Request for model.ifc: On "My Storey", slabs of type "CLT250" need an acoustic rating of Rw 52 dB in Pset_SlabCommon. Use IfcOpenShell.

First a look at what the model holds.

```python
import ifcopenshell
import ifcopenshell.util.element

model = ifcopenshell.open("model.ifc")
print(model.schema)
storey = next(s for s in model.by_type("IfcBuildingStorey") if s.Name == "My Storey")
slabs = [e for e in ifcopenshell.util.element.get_decomposition(storey) if e.is_a("IfcSlab")]
seen = {}
for e in slabs:
    element_type = ifcopenshell.util.element.get_type(e)
    key = (element_type.Name if element_type != e and element_type else None, ifcopenshell.util.element.get_pset(e, "Pset_SlabCommon", "AcousticRating"))
    seen[key] = seen.get(key, 0) + 1
for (name, value), count in sorted(seen.items(), key=str):
    print(count, "x", name, "|", value)
```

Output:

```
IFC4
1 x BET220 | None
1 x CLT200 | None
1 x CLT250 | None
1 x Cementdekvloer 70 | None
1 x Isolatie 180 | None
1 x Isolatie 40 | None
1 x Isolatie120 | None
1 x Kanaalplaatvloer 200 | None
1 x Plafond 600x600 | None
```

```python
import ifcopenshell
import ifcopenshell.api.pset
import ifcopenshell.util.element

model = ifcopenshell.open("model.ifc")

storey = next(s for s in model.by_type("IfcBuildingStorey") if s.Name == "My Storey")
slabs = [e for e in ifcopenshell.util.element.get_decomposition(storey) if e.is_a("IfcSlab")]

count = 0
for e in slabs:
    element_type = ifcopenshell.util.element.get_type(e)
    if element_type in (None, e) or element_type.Name != "CLT250":
        continue
    # add_pset returns the element's existing set when there is one.
    pset = ifcopenshell.api.pset.add_pset(model, product=e, name="Pset_SlabCommon")
    ifcopenshell.api.pset.edit_pset(model, pset=pset, properties={"AcousticRating": "Rw 52 dB"})
    count += 1

print(count, "slabs updated")

model.write("model_edited.ifc")
```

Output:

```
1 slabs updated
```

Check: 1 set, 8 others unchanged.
